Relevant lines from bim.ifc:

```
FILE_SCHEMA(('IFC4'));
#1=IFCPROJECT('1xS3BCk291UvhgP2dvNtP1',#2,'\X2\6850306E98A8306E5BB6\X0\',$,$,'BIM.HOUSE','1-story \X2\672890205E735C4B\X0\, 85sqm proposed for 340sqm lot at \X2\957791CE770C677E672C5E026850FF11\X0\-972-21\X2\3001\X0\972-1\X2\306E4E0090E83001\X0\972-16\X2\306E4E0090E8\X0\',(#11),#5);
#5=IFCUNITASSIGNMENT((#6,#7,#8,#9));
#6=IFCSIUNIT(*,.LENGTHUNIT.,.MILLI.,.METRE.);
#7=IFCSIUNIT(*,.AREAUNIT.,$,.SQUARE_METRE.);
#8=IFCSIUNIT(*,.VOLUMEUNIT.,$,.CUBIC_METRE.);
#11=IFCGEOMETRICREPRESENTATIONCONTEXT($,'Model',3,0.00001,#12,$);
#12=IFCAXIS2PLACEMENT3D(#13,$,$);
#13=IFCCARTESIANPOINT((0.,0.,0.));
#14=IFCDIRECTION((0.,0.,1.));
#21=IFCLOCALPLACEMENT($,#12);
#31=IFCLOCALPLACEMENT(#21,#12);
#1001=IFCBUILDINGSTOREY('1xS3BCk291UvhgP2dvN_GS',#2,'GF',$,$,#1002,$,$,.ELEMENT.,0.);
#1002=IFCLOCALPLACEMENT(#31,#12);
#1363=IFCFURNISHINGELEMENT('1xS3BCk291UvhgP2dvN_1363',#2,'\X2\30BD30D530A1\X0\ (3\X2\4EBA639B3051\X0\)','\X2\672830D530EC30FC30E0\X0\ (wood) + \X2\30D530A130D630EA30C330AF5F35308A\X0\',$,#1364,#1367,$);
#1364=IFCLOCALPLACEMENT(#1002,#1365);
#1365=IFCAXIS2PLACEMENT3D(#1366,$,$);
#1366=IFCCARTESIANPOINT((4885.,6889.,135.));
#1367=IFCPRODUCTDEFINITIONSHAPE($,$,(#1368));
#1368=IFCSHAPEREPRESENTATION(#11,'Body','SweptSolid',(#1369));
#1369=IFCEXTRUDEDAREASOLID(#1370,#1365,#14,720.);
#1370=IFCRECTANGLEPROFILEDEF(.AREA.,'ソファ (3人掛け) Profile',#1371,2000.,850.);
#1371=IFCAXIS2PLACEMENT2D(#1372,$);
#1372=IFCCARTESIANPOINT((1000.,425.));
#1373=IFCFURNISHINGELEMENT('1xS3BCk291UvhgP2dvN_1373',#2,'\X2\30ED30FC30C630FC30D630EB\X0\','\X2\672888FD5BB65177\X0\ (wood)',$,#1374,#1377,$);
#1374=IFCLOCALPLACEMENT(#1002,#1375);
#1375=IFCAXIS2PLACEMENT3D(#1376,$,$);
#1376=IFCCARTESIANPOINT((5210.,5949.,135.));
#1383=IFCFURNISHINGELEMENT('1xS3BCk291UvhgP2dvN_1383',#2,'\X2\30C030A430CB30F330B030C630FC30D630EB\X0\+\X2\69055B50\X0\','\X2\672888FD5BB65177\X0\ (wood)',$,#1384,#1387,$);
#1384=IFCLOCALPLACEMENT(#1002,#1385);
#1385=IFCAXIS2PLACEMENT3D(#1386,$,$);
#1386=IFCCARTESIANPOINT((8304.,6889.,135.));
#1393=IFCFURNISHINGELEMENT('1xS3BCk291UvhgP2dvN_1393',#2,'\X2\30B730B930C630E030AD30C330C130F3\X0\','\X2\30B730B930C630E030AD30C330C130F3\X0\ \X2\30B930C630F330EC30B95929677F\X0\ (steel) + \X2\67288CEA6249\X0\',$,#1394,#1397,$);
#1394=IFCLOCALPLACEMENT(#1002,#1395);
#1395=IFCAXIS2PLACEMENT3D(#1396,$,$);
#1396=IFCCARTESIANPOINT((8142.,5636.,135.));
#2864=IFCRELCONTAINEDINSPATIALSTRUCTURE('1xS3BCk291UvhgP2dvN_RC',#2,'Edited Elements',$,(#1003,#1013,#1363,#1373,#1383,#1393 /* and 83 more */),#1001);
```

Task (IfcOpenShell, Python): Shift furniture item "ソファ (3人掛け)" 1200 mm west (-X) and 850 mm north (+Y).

```python
import ifcopenshell
import ifcopenshell.api.geometry
import ifcopenshell.util.placement

model = ifcopenshell.open("bim.ifc")

item = model.by_guid("1xS3BCk291UvhgP2dvN_1363")
matrix = ifcopenshell.util.placement.get_local_placement(item.ObjectPlacement)
matrix[0, 3] -= 1200.0
matrix[1, 3] += 850.0
ifcopenshell.api.geometry.edit_object_placement(model, product=item, matrix=matrix, is_si=False)

print(ifcopenshell.util.placement.get_local_placement(item.ObjectPlacement).round(3) + 0.0)

model.write("bim-out.ifc")
```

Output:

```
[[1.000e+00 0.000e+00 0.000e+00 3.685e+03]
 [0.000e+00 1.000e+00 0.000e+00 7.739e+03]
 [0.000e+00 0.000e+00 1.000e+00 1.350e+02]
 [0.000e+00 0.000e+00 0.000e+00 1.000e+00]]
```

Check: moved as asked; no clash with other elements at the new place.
